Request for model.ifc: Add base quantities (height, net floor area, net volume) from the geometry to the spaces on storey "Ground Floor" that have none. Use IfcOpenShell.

First a look at what the model holds.

```python
import ifcopenshell
import ifcopenshell.util.element
import ifcopenshell.util.unit

model = ifcopenshell.open("model.ifc")
print(model.schema)
for unit_type in ("LENGTHUNIT", "AREAUNIT", "VOLUMEUNIT"):
    print(unit_type, ifcopenshell.util.unit.calculate_unit_scale(model, unit_type))
storey = next(s for s in model.by_type("IfcBuildingStorey") if s.Name == "Ground Floor")
spaces = [e for e in ifcopenshell.util.element.get_decomposition(storey) if e.is_a("IfcSpace")]
for e in sorted(spaces, key=lambda e: e.id()):
    print(e.id(), e.is_a(), e.Name, list(ifcopenshell.util.element.get_psets(e, qtos_only=True)), sep=" | ")
```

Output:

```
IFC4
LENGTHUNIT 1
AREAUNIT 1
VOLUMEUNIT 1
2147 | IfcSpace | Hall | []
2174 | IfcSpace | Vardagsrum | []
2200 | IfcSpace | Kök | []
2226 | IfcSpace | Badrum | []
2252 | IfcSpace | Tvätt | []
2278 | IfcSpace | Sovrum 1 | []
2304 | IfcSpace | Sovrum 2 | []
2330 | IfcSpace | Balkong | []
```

```python
import ifcopenshell
import ifcopenshell.api.pset
import ifcopenshell.geom
import ifcopenshell.util.element
import ifcopenshell.util.shape
import ifcopenshell.util.unit

model = ifcopenshell.open("model.ifc")
unit_scale = ifcopenshell.util.unit.calculate_unit_scale(model)
area_scale = ifcopenshell.util.unit.calculate_unit_scale(model, "AREAUNIT")
volume_scale = ifcopenshell.util.unit.calculate_unit_scale(model, "VOLUMEUNIT")
settings = ifcopenshell.geom.settings()

storey = next(s for s in model.by_type("IfcBuildingStorey") if s.Name == "Ground Floor")
spaces = [e for e in ifcopenshell.util.element.get_decomposition(storey) if e.is_a("IfcSpace")]

for e in sorted(spaces, key=lambda e: e.id()):
    if ifcopenshell.util.element.get_psets(e, qtos_only=True, should_inherit=False):
        continue
    # Geometry comes back in metres, in the element's own axes.
    shape = ifcopenshell.geom.create_shape(settings, e)
    values = {
        "Height": ifcopenshell.util.shape.get_z(shape.geometry) / unit_scale,
        "NetFloorArea": ifcopenshell.util.shape.get_footprint_area(shape.geometry) / area_scale,
        "NetVolume": ifcopenshell.util.shape.get_volume(shape.geometry) / volume_scale,
    }
    qto = ifcopenshell.api.pset.add_qto(model, product=e, name="Qto_SpaceBaseQuantities")
    ifcopenshell.api.pset.edit_qto(model, qto=qto, properties=values)
    print(e.id(), {k: round(v, 3) for k, v in values.items()})

model.write("model_edited.ifc")
```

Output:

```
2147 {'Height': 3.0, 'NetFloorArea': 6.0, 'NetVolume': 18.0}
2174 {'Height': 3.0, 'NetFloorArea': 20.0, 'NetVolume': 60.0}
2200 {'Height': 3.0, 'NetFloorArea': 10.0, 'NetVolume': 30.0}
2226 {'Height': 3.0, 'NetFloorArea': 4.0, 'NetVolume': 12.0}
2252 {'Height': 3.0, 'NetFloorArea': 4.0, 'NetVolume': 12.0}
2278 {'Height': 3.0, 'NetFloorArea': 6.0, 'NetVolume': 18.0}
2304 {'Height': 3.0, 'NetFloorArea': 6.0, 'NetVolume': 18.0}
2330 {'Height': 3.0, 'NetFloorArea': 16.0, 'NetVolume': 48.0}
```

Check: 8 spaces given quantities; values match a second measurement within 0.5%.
